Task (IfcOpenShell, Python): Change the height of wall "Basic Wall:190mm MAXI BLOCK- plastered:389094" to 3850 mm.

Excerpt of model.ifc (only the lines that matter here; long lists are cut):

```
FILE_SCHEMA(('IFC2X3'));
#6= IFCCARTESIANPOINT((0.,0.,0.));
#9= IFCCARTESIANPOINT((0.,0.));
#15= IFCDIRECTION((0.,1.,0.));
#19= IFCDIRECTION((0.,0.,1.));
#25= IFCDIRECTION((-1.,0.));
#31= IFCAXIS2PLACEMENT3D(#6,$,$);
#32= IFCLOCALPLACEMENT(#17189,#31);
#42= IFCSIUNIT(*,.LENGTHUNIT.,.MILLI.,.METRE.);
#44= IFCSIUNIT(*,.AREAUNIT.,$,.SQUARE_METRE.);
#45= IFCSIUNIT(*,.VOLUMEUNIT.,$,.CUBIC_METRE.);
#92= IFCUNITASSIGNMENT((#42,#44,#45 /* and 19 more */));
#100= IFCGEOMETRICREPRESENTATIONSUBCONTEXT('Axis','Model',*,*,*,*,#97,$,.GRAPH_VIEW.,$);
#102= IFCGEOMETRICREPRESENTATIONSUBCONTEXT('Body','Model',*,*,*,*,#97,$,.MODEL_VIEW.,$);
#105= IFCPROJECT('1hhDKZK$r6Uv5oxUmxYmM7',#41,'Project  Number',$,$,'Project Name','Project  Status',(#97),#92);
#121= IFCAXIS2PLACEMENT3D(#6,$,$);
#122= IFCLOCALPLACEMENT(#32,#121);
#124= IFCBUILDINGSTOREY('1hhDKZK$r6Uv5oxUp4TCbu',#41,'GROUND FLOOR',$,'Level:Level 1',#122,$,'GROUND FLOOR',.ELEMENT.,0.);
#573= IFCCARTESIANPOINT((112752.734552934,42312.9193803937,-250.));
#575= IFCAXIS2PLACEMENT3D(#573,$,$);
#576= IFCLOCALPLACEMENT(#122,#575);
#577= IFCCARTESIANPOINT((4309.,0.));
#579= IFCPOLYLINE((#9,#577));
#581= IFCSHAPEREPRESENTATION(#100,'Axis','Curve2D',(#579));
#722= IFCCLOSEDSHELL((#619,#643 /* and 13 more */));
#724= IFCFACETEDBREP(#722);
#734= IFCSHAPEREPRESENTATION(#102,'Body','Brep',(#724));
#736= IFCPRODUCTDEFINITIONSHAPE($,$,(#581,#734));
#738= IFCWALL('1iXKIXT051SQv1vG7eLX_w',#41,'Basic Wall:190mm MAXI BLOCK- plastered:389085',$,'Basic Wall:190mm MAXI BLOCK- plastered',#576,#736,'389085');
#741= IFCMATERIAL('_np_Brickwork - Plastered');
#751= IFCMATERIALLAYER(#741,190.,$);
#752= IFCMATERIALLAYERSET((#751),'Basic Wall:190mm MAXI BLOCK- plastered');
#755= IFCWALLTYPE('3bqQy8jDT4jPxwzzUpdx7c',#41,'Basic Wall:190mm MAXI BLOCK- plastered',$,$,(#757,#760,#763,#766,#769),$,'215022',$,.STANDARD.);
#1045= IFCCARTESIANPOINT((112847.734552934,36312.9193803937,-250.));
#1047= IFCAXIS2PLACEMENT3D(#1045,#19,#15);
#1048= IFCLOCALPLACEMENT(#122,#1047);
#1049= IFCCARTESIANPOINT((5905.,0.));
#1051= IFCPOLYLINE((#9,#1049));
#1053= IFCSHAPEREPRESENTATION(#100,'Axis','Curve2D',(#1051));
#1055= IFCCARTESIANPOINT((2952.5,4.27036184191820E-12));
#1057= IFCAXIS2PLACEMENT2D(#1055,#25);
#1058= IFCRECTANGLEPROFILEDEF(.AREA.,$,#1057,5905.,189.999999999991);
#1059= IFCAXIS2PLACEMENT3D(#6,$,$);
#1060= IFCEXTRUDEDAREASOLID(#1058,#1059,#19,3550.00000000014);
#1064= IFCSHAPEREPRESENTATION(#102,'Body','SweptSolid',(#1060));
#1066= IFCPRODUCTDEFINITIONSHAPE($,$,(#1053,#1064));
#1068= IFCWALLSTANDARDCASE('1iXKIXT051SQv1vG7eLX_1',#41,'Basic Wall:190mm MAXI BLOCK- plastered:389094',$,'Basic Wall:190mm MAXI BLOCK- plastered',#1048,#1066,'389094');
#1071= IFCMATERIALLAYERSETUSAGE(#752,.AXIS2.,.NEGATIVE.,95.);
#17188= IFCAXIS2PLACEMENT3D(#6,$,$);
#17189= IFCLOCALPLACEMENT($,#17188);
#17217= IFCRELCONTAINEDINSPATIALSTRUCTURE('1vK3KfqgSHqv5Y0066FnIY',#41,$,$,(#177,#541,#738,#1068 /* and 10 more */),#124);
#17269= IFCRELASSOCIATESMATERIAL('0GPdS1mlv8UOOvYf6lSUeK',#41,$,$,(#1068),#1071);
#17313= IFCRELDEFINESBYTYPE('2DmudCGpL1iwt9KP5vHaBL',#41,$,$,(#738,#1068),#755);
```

```python
import ifcopenshell
import ifcopenshell.geom
import ifcopenshell.util.representation
import ifcopenshell.util.shape
import ifcopenshell.util.unit

model = ifcopenshell.open("model.ifc")
unit_scale = ifcopenshell.util.unit.calculate_unit_scale(model)
settings = ifcopenshell.geom.settings()


def volume(element):
    """Net volume in cubic metres, openings subtracted."""
    shape = ifcopenshell.geom.create_shape(settings, element)
    return ifcopenshell.util.shape.get_volume(shape.geometry)


wall = model.by_guid("1iXKIXT051SQv1vG7eLX_1")
before = volume(wall)

body = ifcopenshell.util.representation.get_representation(wall, "Model", "Body")
solid = body.Items[0]
old_height = solid.Depth
solid.Depth = 3.85 / unit_scale
after = volume(wall)

print(f"height {old_height:g} -> {solid.Depth:g}, volume {before:.3f} -> {after:.3f} m3")

model.write("model_rev.ifc")
```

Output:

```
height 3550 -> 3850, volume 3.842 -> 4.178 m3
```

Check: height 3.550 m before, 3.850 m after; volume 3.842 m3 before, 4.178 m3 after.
